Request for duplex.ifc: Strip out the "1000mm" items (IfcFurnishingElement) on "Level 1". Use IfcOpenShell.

First a look at what the model holds.

```python
import ifcopenshell
import ifcopenshell.util.element

model = ifcopenshell.open("duplex.ifc")
print(model.schema)
storey = next(s for s in model.by_type("IfcBuildingStorey") if s.Name == "Level 1")
furniture = [e for e in ifcopenshell.util.element.get_decomposition(storey) if e.is_a("IfcFurnishingElement")]
seen = {}
for e in furniture:
    element_type = ifcopenshell.util.element.get_type(e)
    name = element_type.Name if element_type not in (None, e) else None
    seen[name] = seen.get(name, 0) + 1
for name, count in sorted(seen.items(), key=str):
    print(count, "x", name)
```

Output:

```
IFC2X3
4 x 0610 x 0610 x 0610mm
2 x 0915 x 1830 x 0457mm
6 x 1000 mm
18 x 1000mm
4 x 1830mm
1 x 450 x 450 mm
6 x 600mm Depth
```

```python
import ifcopenshell
import ifcopenshell.api.root
import ifcopenshell.util.element

model = ifcopenshell.open("duplex.ifc")

storey = next(s for s in model.by_type("IfcBuildingStorey") if s.Name == "Level 1")
furniture = [e for e in ifcopenshell.util.element.get_decomposition(storey) if e.is_a("IfcFurnishingElement")]
targets = [e for e in furniture if (t := ifcopenshell.util.element.get_type(e)) not in (None, e) and t.Name == "1000mm"]

for e in targets:
    ifcopenshell.api.root.remove_product(model, product=e)
print(len(targets), "removed")

model.write("duplex-out.ifc")
```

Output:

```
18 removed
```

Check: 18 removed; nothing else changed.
